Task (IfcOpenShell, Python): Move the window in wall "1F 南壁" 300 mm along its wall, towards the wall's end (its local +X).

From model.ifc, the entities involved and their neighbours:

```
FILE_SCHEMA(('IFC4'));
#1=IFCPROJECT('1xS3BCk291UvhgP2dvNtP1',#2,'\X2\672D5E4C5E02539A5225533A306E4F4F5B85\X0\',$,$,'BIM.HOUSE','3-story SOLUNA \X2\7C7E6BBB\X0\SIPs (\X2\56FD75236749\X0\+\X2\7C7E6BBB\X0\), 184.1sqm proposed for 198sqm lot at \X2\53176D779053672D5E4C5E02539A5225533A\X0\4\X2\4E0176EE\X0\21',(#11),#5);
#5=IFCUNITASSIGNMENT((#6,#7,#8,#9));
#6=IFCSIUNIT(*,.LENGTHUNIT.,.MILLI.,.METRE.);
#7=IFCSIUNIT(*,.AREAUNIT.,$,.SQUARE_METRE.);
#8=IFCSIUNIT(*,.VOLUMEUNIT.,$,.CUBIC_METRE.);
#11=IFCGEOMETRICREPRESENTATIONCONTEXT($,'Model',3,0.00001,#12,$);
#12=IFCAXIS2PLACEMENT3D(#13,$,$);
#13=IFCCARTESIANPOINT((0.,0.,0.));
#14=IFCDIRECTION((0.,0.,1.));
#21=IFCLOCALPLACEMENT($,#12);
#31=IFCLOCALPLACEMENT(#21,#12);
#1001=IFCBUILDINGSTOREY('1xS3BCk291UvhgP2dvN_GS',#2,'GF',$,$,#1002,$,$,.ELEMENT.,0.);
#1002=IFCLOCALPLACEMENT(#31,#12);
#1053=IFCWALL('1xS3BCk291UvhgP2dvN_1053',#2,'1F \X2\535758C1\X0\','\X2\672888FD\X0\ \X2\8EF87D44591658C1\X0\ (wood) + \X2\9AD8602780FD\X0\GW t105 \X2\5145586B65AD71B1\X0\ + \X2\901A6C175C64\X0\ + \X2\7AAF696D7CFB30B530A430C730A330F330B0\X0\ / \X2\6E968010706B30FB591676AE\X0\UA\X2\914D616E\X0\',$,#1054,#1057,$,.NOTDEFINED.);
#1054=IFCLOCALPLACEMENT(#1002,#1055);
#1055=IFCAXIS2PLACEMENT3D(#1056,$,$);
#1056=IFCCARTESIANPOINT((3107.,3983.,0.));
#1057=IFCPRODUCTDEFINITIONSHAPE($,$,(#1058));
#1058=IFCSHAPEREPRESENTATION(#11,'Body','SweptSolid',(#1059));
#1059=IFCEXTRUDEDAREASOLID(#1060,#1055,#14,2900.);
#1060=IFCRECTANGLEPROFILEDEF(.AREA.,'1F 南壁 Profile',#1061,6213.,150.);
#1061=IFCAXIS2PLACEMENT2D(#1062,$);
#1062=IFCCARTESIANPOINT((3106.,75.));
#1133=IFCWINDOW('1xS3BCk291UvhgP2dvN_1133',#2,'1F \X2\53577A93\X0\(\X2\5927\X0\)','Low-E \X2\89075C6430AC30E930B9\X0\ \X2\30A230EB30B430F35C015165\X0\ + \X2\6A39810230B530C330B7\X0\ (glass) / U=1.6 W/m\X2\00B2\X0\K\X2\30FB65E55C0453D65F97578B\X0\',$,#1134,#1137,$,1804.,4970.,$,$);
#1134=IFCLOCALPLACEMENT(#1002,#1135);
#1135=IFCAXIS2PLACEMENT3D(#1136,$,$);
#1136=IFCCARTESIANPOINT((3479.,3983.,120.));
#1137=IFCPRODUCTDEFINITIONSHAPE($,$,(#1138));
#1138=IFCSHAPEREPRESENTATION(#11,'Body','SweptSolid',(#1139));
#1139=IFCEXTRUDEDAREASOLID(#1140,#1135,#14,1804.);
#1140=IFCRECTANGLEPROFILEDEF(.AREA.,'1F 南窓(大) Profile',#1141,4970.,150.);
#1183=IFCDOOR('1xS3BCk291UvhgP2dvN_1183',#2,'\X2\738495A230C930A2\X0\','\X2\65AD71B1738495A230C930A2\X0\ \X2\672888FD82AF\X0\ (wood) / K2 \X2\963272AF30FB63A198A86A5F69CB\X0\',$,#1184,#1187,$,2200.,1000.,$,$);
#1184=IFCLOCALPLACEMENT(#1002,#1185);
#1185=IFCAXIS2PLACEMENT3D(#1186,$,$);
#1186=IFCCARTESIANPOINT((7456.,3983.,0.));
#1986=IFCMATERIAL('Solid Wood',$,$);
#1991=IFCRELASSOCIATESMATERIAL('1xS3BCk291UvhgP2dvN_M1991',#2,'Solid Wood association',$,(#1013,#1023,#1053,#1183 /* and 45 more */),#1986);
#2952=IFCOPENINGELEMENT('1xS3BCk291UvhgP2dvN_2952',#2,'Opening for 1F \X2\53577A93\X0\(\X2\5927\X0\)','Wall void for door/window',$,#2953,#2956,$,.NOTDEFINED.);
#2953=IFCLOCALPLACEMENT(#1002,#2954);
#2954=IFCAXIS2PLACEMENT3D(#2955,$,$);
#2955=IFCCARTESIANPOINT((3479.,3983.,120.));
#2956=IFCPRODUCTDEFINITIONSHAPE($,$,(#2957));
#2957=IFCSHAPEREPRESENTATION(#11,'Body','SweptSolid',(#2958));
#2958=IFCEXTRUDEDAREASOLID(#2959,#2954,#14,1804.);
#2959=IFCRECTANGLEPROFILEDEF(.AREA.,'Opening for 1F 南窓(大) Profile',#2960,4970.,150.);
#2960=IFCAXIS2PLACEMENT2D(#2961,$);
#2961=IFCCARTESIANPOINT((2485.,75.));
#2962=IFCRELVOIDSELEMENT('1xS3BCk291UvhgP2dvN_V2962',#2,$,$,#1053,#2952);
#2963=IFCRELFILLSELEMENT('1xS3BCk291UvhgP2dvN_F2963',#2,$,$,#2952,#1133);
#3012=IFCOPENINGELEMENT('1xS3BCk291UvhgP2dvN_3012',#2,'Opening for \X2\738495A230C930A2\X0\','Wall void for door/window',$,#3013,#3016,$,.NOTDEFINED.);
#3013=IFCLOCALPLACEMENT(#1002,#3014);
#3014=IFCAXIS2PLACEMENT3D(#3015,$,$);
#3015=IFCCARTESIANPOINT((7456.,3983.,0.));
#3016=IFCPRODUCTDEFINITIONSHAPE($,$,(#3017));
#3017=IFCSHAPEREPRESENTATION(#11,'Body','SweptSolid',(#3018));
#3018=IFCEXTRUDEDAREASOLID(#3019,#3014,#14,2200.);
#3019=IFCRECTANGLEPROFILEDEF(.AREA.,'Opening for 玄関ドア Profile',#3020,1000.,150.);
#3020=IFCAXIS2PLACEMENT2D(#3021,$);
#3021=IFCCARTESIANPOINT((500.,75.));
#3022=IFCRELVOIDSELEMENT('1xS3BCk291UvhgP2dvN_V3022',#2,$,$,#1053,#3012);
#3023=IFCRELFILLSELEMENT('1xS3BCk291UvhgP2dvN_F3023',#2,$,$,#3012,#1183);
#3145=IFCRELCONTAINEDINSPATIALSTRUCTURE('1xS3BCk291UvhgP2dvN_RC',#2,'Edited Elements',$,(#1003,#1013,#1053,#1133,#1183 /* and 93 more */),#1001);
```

```python
import ifcopenshell
import ifcopenshell.api.geometry
import ifcopenshell.util.placement
import ifcopenshell.util.unit

model = ifcopenshell.open("model.ifc")
unit_scale = ifcopenshell.util.unit.calculate_unit_scale(model)

window = model.by_guid("1xS3BCk291UvhgP2dvN_1133")
opening = window.FillsVoids[0].RelatingOpeningElement
wall = opening.VoidsElements[0].RelatingBuildingElement

wall_matrix = ifcopenshell.util.placement.get_local_placement(wall.ObjectPlacement)
shift = wall_matrix[:3, 0] * 0.3 / unit_scale
before = ifcopenshell.util.placement.get_local_placement(window.ObjectPlacement)[:3, 3].copy()

# The window is not placed relative to its opening, so move both.
for product in (opening, window):
    matrix = ifcopenshell.util.placement.get_local_placement(product.ObjectPlacement)
    matrix[:3, 3] += shift
    ifcopenshell.api.geometry.edit_object_placement(model, product=product, matrix=matrix, is_si=False)

after = ifcopenshell.util.placement.get_local_placement(window.ObjectPlacement)[:3, 3]
print("window moved by", (after - before).round(3) + 0.0)

model.write("model-out.ifc")
```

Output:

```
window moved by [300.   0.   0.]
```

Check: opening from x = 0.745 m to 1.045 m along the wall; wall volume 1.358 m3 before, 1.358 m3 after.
